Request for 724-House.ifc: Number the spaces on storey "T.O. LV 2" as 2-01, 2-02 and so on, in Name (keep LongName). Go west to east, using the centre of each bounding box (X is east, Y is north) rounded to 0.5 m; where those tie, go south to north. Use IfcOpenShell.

First a look at what the model holds.

```python
import ifcopenshell
import ifcopenshell.util.element
import ifcopenshell.util.placement

model = ifcopenshell.open("724-House.ifc")
print(model.schema)
storey = next(s for s in model.by_type("IfcBuildingStorey") if s.Name == "T.O. LV 2")
spaces = [e for e in ifcopenshell.util.element.get_decomposition(storey) if e.is_a("IfcSpace")]
for e in sorted(spaces, key=lambda e: e.id()):
    origin = ifcopenshell.util.placement.get_local_placement(e.ObjectPlacement)[:3, 3]
    print(e.id(), e.Name, e.LongName, origin.round(2) + 0.0, sep=" | ")
```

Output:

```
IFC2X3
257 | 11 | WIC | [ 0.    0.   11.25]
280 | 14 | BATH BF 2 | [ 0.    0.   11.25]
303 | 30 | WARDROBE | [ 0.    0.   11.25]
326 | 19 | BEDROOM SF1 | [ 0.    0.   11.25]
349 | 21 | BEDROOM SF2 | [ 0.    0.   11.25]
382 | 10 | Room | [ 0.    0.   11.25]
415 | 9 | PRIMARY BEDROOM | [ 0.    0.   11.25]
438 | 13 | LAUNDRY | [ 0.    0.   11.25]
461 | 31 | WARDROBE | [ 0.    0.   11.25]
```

```python
import ifcopenshell
import ifcopenshell.geom
import ifcopenshell.util.element
import ifcopenshell.util.shape

model = ifcopenshell.open("724-House.ifc")
settings = ifcopenshell.geom.settings()
settings.set("use-world-coords", True)


def centre(element):
    shape = ifcopenshell.geom.create_shape(settings, element)
    return ifcopenshell.util.shape.get_bbox_centroid(shape.geometry)


storey = next(s for s in model.by_type("IfcBuildingStorey") if s.Name == "T.O. LV 2")
spaces = [e for e in ifcopenshell.util.element.get_decomposition(storey) if e.is_a("IfcSpace")]

# Insertion points can sit at a corner or the storey origin, so sort by the geometry (in metres).
centres = {e: centre(e) for e in spaces}
spaces.sort(key=lambda e: (round(centres[e][0] / 0.5), centres[e][1]))

for i, e in enumerate(spaces, start=1):
    number = f"2-{i:02d}"
    e.Name = number
    print(e.id(), number)

model.write("724-House-out.ifc")
```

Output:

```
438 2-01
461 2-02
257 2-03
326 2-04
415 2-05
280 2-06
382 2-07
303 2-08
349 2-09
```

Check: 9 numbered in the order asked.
